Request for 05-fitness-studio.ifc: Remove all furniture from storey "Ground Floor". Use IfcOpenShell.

First a look at what the model holds.

```python
import ifcopenshell
import ifcopenshell.util.element

model = ifcopenshell.open("05-fitness-studio.ifc")
print(model.schema)
storey = next(s for s in model.by_type("IfcBuildingStorey") if s.Name == "Ground Floor")
furniture = [e for e in ifcopenshell.util.element.get_decomposition(storey) if e.is_a("IfcFurnishingElement")]
seen = {}
for e in furniture:
    element_type = ifcopenshell.util.element.get_type(e)
    name = element_type.Name if element_type not in (None, e) else None
    seen[name] = seen.get(name, 0) + 1
for name, count in sorted(seen.items(), key=str):
    print(count, "x", name)
```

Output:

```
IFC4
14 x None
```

```python
import ifcopenshell
import ifcopenshell.api.root
import ifcopenshell.util.element

model = ifcopenshell.open("05-fitness-studio.ifc")

storey = next(s for s in model.by_type("IfcBuildingStorey") if s.Name == "Ground Floor")
furniture = [e for e in ifcopenshell.util.element.get_decomposition(storey) if e.is_a("IfcFurnishingElement")]

for e in furniture:
    ifcopenshell.api.root.remove_product(model, product=e)
print(len(furniture), "removed")

model.write("05-fitness-studio_edited.ifc")
```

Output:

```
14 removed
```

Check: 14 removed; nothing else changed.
